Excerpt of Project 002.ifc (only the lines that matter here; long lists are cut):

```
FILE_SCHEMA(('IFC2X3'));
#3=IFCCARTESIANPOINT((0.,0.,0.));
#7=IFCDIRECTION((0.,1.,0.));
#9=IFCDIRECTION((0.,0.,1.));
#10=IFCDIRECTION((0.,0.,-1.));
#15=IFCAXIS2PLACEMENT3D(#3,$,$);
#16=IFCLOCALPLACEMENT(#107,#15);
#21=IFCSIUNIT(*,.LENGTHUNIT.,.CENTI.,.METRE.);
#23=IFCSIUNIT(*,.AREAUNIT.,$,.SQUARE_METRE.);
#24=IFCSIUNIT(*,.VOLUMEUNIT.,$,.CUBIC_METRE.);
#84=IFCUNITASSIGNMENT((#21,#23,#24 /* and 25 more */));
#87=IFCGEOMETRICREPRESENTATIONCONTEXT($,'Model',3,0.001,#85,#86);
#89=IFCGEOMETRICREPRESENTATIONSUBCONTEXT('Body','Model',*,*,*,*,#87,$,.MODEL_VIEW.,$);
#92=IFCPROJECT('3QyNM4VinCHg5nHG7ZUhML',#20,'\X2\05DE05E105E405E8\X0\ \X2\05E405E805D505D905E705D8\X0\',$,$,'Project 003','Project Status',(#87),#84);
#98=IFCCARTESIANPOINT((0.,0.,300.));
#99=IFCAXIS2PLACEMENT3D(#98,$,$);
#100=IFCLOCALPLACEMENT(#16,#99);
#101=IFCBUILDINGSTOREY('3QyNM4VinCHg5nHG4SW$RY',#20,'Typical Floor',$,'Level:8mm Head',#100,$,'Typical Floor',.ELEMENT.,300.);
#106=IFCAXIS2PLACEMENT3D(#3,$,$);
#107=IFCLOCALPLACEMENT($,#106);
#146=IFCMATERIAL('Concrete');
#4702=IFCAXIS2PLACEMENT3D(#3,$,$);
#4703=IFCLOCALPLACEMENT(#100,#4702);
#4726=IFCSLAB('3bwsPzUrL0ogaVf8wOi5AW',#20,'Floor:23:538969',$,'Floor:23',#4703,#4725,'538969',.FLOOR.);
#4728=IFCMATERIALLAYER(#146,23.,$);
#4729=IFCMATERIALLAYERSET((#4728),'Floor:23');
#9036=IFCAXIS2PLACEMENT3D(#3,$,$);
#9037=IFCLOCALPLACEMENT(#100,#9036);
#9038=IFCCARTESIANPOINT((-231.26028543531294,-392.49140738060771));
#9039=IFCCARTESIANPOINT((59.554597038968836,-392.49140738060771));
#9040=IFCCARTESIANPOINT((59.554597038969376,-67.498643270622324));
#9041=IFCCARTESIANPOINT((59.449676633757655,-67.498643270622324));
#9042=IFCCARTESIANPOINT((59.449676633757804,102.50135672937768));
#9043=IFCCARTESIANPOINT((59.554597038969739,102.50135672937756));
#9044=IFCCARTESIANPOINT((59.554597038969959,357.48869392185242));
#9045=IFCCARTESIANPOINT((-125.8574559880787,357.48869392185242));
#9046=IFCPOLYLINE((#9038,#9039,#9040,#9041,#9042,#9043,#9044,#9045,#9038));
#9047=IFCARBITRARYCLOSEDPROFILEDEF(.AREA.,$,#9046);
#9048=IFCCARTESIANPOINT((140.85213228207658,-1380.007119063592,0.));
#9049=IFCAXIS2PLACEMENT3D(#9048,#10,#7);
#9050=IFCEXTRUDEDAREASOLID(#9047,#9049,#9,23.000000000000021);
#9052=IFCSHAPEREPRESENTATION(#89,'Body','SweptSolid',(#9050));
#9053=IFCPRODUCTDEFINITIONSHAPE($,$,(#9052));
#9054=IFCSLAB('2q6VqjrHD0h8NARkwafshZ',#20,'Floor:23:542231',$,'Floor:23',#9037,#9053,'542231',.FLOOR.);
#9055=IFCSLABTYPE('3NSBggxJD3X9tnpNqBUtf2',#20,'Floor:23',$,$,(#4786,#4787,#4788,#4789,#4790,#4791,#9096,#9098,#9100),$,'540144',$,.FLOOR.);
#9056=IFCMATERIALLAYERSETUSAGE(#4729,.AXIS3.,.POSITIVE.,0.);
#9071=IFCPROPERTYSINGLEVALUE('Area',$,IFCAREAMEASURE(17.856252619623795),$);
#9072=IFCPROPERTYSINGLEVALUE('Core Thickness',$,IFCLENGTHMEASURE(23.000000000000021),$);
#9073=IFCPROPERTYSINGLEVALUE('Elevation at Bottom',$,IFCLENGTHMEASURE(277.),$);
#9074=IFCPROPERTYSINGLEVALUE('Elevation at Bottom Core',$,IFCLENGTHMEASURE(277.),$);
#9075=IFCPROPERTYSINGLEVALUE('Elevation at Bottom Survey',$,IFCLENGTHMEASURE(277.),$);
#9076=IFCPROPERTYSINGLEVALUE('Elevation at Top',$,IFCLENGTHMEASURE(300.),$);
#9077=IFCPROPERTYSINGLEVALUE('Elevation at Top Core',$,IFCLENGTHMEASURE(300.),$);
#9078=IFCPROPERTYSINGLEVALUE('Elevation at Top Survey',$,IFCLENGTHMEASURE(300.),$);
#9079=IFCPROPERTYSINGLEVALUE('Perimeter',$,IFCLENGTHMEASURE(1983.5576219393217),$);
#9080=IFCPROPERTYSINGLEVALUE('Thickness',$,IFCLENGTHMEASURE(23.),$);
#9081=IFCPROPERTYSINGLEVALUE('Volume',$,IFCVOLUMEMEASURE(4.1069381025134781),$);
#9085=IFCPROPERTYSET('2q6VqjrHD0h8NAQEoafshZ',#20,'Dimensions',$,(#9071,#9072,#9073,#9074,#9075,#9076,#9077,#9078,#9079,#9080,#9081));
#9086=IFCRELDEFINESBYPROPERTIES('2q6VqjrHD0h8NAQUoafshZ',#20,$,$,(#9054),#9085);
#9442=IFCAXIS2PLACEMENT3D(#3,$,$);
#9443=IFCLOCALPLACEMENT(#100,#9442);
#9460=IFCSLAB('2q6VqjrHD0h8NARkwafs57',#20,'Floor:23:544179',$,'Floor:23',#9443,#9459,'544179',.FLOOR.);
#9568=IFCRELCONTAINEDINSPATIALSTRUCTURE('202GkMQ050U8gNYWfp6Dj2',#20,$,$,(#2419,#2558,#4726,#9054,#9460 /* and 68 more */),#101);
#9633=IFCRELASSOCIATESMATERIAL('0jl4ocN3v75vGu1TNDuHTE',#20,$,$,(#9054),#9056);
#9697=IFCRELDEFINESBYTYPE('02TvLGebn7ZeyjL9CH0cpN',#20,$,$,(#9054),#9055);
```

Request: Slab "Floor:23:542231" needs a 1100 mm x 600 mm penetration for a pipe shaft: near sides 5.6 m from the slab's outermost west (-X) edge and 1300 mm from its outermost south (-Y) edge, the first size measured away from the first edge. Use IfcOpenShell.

```python
import numpy as np
import ifcopenshell
import ifcopenshell.api.feature
import ifcopenshell.api.geometry
import ifcopenshell.api.pset
import ifcopenshell.api.root
import ifcopenshell.geom
import ifcopenshell.util.element
import ifcopenshell.util.placement
import ifcopenshell.util.representation
import ifcopenshell.util.shape
import ifcopenshell.util.unit

model = ifcopenshell.open("Project 002.ifc")
unit_scale = ifcopenshell.util.unit.calculate_unit_scale(model)
area_scale = ifcopenshell.util.unit.calculate_unit_scale(model, "AREAUNIT")
volume_scale = ifcopenshell.util.unit.calculate_unit_scale(model, "VOLUMEUNIT")
settings = ifcopenshell.geom.settings()


def volume(element):
    """Net volume in cubic metres, openings subtracted."""
    shape = ifcopenshell.geom.create_shape(settings, element)
    return ifcopenshell.util.shape.get_volume(shape.geometry)


slab = model.by_id(9054)
before = volume(slab)

# Extent in the slab's own axes, in metres. The edges named are its -X and -Y sides.
slab_shape = ifcopenshell.geom.create_shape(settings, slab)
vertices = ifcopenshell.util.shape.get_vertices(slab_shape.geometry)
x_min, y_min, bottom = vertices.min(axis=0)
top = vertices[:, 2].max()

opening = ifcopenshell.api.root.create_entity(model, ifc_class="IfcOpeningElement", name="Pipe shaft opening")
context = ifcopenshell.util.representation.get_context(model, "Model", "Body", "MODEL_VIEW")
width, depth = 1.1, 0.6
outline = [(0.0, 0.0), (width, 0.0), (width, depth), (0.0, depth), (0.0, 0.0)]
# Overshoot both faces by 50 mm so the cut is clean.
shape = ifcopenshell.api.geometry.add_slab_representation(
    model, context=context, depth=top - bottom + 0.1, polyline=outline
)
ifcopenshell.api.geometry.assign_representation(model, product=opening, representation=shape)

matrix = ifcopenshell.util.placement.get_local_placement(slab.ObjectPlacement)
matrix[:, 3] = matrix @ np.append(np.array([x_min + 5.6, y_min + 1.3, bottom - 0.05]) / unit_scale, 1.0)
ifcopenshell.api.geometry.edit_object_placement(model, product=opening, matrix=matrix, is_si=False)
ifcopenshell.api.feature.add_feature(model, feature=opening, element=slab)

after = volume(slab)

# Update the slab's stored quantities.
pset = model.by_id(ifcopenshell.util.element.get_pset(slab, "Dimensions", should_inherit=False)["id"])
ifcopenshell.api.pset.edit_pset(model, pset=pset, properties={
    "Area": model.create_entity("IfcAreaMeasure", after / (top - bottom) / area_scale),
    "Volume": model.create_entity("IfcVolumeMeasure", after / volume_scale),
})

print(f"slab volume {before:.3f} -> {after:.3f} m3")

model.write("Project 002_rev.ifc")
```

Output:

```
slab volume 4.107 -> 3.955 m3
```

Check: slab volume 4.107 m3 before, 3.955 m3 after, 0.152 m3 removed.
